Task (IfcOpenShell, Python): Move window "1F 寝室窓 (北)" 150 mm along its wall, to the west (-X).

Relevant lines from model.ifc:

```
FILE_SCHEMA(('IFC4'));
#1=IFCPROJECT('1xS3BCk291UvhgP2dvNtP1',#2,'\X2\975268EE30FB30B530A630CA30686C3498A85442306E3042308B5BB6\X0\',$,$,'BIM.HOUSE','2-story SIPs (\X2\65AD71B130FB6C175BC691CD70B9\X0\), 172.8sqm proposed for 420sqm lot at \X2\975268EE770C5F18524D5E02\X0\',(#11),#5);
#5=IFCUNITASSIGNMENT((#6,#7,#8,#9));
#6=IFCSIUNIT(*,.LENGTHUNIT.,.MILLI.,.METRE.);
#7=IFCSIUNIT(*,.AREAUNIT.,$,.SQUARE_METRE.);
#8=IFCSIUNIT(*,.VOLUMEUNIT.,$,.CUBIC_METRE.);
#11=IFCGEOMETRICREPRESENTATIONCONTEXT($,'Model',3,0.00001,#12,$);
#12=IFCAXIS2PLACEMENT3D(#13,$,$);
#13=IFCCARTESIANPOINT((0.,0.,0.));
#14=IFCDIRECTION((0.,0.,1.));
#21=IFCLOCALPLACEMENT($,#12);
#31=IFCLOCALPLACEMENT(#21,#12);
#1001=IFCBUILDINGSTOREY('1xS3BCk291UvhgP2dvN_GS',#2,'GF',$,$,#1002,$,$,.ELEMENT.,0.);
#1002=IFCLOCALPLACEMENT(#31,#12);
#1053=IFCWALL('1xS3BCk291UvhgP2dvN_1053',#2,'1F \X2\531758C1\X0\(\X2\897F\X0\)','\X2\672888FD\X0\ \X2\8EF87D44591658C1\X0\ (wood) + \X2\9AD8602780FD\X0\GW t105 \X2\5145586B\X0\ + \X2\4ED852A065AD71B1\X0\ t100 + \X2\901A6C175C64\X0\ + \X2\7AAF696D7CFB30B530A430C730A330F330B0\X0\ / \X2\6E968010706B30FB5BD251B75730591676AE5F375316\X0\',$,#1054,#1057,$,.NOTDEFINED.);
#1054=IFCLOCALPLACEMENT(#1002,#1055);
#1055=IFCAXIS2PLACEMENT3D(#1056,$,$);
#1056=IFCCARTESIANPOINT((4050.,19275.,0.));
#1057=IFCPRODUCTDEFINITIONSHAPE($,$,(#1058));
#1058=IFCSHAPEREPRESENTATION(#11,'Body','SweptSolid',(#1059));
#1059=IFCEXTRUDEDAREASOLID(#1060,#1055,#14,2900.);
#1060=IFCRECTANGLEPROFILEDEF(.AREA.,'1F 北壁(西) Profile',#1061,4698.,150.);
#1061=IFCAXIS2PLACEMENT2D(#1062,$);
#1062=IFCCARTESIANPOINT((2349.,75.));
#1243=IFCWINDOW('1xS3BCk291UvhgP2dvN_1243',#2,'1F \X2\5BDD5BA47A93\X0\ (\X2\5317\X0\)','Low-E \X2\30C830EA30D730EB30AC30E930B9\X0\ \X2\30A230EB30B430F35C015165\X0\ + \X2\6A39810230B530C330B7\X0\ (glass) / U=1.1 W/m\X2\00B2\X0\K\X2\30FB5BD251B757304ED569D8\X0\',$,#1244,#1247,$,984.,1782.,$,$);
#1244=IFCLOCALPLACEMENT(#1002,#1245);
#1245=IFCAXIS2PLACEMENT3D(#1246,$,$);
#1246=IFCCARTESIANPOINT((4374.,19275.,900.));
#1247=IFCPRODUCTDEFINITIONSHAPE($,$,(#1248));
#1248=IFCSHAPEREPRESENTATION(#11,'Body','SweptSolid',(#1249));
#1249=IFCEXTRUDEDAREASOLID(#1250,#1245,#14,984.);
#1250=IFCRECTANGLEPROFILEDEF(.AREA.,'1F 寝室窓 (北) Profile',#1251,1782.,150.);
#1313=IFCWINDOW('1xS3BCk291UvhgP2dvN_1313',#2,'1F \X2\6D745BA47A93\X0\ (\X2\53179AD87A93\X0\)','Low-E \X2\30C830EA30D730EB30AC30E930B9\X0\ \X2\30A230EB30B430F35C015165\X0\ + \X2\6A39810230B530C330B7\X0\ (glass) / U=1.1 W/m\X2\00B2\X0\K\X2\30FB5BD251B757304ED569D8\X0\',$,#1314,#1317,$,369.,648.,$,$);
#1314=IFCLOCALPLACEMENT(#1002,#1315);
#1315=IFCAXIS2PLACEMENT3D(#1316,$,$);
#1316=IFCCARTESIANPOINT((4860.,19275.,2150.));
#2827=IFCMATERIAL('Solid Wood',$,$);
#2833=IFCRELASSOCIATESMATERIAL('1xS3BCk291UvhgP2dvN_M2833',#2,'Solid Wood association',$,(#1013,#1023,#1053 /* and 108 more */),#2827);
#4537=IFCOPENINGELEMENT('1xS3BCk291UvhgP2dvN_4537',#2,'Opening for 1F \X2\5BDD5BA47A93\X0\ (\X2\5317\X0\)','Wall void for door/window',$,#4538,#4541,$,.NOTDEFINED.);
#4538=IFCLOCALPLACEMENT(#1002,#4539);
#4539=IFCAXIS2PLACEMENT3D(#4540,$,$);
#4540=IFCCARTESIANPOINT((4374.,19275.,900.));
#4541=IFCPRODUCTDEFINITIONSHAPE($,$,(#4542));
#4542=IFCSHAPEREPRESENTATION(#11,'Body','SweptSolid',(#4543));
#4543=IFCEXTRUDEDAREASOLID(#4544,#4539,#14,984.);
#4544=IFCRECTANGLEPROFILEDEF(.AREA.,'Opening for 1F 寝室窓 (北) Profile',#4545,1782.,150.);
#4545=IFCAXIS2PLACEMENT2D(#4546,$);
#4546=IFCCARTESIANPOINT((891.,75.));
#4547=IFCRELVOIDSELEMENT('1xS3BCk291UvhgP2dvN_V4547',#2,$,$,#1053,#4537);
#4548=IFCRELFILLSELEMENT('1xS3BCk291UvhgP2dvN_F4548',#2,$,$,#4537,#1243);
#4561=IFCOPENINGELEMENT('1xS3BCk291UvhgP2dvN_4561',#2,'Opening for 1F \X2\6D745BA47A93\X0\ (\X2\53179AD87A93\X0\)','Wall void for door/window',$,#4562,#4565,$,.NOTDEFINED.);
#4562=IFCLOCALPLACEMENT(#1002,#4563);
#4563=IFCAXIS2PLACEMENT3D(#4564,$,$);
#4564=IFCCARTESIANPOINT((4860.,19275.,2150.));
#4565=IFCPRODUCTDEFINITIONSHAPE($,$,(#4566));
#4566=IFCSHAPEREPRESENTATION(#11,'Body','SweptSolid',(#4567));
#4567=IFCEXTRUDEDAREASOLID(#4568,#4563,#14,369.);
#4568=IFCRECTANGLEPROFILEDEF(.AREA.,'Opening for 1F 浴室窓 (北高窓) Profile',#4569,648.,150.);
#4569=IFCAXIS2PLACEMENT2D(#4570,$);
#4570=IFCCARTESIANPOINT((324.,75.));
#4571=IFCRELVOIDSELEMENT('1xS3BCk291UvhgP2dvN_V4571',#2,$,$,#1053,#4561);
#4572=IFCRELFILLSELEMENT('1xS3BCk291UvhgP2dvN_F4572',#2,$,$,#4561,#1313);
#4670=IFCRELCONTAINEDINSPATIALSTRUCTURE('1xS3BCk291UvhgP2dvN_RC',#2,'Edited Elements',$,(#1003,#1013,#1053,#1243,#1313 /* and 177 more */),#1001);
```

```python
import ifcopenshell
import ifcopenshell.api.geometry
import ifcopenshell.util.placement

model = ifcopenshell.open("model.ifc")

window = model.by_guid("1xS3BCk291UvhgP2dvN_1243")
opening = window.FillsVoids[0].RelatingOpeningElement
wall = opening.VoidsElements[0].RelatingBuildingElement

wall_matrix = ifcopenshell.util.placement.get_local_placement(wall.ObjectPlacement)
shift = wall_matrix[:3, 0] * -150.0
before = ifcopenshell.util.placement.get_local_placement(window.ObjectPlacement)[:3, 3].copy()

# The window is not placed relative to its opening, so move both.
for product in (opening, window):
    matrix = ifcopenshell.util.placement.get_local_placement(product.ObjectPlacement)
    matrix[:3, 3] += shift
    ifcopenshell.api.geometry.edit_object_placement(model, product=product, matrix=matrix, is_si=False)

after = ifcopenshell.util.placement.get_local_placement(window.ObjectPlacement)[:3, 3]
print("window moved by", (after - before).round(3) + 0.0)

model.write("model_rev.ifc")
```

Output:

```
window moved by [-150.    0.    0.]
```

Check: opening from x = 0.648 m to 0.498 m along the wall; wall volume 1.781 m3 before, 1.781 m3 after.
